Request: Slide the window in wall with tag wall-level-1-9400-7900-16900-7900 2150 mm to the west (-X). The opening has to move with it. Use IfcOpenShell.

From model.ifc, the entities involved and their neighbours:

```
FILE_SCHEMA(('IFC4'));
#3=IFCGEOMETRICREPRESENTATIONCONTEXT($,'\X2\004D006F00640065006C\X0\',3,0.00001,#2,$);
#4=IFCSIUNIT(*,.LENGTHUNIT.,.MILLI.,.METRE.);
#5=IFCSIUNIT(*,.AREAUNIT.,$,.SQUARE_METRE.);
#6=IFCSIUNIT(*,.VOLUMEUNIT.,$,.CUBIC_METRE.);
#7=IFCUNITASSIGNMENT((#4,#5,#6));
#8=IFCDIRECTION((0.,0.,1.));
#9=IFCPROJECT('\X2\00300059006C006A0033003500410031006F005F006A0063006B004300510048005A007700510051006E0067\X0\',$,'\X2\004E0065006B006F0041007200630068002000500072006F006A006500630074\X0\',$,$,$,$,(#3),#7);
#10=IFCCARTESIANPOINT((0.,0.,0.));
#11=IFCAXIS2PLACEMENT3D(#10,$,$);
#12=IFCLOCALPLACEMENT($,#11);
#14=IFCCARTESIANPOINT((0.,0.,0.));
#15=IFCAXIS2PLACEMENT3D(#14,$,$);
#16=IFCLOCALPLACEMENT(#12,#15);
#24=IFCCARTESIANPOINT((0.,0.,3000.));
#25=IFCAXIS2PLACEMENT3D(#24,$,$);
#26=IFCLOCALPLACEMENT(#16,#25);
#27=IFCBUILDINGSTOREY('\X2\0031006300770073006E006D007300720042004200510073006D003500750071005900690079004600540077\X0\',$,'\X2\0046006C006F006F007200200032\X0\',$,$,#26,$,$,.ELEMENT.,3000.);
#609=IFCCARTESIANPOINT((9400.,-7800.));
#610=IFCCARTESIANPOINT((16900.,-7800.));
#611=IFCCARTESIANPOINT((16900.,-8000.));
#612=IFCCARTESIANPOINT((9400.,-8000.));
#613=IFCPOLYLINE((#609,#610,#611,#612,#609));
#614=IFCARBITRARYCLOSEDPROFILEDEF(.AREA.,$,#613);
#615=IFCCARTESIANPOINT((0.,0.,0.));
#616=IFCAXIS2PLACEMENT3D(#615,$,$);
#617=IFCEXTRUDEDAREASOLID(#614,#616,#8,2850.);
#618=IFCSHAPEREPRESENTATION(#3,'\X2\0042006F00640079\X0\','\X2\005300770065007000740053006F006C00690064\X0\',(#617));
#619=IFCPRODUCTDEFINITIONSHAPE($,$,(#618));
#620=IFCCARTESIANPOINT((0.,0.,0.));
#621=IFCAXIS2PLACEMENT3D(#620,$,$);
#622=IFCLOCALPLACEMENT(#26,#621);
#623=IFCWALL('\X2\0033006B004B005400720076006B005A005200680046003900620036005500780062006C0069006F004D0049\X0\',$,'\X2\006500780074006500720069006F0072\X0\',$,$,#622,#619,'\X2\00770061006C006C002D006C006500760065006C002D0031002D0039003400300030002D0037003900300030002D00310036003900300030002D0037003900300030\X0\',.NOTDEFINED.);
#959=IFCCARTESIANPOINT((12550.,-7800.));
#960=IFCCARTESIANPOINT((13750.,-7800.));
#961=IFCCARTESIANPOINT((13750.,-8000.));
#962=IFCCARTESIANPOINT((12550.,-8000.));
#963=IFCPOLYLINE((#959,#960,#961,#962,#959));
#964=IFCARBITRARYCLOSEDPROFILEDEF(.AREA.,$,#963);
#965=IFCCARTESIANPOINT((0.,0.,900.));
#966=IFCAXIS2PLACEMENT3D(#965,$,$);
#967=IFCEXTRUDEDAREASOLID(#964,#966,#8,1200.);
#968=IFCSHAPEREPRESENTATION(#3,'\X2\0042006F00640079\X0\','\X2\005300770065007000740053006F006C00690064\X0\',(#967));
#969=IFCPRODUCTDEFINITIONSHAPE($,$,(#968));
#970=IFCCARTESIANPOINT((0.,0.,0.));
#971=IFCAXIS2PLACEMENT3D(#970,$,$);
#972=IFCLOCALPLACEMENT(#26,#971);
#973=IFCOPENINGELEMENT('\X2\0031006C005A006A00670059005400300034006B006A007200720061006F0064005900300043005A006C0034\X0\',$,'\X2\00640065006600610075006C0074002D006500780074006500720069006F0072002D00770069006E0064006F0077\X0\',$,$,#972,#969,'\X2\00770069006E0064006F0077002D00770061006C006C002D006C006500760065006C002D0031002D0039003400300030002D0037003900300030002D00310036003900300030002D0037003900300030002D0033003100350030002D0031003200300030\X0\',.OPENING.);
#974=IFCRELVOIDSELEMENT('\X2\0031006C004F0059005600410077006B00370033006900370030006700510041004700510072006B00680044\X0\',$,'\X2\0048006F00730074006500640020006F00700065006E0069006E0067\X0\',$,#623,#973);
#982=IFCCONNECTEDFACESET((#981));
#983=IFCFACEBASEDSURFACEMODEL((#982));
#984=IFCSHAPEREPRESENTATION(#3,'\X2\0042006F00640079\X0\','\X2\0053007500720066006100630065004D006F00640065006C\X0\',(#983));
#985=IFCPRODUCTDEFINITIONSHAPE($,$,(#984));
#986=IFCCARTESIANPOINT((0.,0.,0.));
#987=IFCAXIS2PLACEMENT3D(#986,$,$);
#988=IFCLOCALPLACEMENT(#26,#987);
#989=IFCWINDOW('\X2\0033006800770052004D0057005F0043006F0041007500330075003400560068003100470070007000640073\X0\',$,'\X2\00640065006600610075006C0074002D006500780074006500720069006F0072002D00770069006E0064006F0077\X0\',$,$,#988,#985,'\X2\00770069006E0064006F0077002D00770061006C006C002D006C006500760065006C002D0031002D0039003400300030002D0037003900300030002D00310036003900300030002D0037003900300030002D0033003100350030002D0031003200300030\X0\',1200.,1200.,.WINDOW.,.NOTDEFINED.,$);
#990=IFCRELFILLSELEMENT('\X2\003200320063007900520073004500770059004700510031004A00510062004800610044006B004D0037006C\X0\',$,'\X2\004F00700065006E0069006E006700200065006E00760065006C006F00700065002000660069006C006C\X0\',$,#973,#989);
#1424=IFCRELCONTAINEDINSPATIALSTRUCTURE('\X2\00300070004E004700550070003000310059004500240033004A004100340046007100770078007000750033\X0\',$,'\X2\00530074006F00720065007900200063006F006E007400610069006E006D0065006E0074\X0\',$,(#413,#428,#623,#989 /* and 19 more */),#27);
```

```python
import ifcopenshell
import ifcopenshell.api.geometry
import ifcopenshell.util.placement
import ifcopenshell.util.unit

model = ifcopenshell.open("model.ifc")
unit_scale = ifcopenshell.util.unit.calculate_unit_scale(model)

window = model.by_id(989)
opening = window.FillsVoids[0].RelatingOpeningElement
wall = opening.VoidsElements[0].RelatingBuildingElement

wall_matrix = ifcopenshell.util.placement.get_local_placement(wall.ObjectPlacement)
shift = wall_matrix[:3, 0] * -2.15 / unit_scale
before = ifcopenshell.util.placement.get_local_placement(window.ObjectPlacement)[:3, 3].copy()

# The window is not placed relative to its opening, so move both.
for product in (opening, window):
    matrix = ifcopenshell.util.placement.get_local_placement(product.ObjectPlacement)
    matrix[:3, 3] += shift
    ifcopenshell.api.geometry.edit_object_placement(model, product=product, matrix=matrix, is_si=False)

after = ifcopenshell.util.placement.get_local_placement(window.ObjectPlacement)[:3, 3]
print("window moved by", (after - before).round(3) + 0.0)

model.write("model-out.ifc")
```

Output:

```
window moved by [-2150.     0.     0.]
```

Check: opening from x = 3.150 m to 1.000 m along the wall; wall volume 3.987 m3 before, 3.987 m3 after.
